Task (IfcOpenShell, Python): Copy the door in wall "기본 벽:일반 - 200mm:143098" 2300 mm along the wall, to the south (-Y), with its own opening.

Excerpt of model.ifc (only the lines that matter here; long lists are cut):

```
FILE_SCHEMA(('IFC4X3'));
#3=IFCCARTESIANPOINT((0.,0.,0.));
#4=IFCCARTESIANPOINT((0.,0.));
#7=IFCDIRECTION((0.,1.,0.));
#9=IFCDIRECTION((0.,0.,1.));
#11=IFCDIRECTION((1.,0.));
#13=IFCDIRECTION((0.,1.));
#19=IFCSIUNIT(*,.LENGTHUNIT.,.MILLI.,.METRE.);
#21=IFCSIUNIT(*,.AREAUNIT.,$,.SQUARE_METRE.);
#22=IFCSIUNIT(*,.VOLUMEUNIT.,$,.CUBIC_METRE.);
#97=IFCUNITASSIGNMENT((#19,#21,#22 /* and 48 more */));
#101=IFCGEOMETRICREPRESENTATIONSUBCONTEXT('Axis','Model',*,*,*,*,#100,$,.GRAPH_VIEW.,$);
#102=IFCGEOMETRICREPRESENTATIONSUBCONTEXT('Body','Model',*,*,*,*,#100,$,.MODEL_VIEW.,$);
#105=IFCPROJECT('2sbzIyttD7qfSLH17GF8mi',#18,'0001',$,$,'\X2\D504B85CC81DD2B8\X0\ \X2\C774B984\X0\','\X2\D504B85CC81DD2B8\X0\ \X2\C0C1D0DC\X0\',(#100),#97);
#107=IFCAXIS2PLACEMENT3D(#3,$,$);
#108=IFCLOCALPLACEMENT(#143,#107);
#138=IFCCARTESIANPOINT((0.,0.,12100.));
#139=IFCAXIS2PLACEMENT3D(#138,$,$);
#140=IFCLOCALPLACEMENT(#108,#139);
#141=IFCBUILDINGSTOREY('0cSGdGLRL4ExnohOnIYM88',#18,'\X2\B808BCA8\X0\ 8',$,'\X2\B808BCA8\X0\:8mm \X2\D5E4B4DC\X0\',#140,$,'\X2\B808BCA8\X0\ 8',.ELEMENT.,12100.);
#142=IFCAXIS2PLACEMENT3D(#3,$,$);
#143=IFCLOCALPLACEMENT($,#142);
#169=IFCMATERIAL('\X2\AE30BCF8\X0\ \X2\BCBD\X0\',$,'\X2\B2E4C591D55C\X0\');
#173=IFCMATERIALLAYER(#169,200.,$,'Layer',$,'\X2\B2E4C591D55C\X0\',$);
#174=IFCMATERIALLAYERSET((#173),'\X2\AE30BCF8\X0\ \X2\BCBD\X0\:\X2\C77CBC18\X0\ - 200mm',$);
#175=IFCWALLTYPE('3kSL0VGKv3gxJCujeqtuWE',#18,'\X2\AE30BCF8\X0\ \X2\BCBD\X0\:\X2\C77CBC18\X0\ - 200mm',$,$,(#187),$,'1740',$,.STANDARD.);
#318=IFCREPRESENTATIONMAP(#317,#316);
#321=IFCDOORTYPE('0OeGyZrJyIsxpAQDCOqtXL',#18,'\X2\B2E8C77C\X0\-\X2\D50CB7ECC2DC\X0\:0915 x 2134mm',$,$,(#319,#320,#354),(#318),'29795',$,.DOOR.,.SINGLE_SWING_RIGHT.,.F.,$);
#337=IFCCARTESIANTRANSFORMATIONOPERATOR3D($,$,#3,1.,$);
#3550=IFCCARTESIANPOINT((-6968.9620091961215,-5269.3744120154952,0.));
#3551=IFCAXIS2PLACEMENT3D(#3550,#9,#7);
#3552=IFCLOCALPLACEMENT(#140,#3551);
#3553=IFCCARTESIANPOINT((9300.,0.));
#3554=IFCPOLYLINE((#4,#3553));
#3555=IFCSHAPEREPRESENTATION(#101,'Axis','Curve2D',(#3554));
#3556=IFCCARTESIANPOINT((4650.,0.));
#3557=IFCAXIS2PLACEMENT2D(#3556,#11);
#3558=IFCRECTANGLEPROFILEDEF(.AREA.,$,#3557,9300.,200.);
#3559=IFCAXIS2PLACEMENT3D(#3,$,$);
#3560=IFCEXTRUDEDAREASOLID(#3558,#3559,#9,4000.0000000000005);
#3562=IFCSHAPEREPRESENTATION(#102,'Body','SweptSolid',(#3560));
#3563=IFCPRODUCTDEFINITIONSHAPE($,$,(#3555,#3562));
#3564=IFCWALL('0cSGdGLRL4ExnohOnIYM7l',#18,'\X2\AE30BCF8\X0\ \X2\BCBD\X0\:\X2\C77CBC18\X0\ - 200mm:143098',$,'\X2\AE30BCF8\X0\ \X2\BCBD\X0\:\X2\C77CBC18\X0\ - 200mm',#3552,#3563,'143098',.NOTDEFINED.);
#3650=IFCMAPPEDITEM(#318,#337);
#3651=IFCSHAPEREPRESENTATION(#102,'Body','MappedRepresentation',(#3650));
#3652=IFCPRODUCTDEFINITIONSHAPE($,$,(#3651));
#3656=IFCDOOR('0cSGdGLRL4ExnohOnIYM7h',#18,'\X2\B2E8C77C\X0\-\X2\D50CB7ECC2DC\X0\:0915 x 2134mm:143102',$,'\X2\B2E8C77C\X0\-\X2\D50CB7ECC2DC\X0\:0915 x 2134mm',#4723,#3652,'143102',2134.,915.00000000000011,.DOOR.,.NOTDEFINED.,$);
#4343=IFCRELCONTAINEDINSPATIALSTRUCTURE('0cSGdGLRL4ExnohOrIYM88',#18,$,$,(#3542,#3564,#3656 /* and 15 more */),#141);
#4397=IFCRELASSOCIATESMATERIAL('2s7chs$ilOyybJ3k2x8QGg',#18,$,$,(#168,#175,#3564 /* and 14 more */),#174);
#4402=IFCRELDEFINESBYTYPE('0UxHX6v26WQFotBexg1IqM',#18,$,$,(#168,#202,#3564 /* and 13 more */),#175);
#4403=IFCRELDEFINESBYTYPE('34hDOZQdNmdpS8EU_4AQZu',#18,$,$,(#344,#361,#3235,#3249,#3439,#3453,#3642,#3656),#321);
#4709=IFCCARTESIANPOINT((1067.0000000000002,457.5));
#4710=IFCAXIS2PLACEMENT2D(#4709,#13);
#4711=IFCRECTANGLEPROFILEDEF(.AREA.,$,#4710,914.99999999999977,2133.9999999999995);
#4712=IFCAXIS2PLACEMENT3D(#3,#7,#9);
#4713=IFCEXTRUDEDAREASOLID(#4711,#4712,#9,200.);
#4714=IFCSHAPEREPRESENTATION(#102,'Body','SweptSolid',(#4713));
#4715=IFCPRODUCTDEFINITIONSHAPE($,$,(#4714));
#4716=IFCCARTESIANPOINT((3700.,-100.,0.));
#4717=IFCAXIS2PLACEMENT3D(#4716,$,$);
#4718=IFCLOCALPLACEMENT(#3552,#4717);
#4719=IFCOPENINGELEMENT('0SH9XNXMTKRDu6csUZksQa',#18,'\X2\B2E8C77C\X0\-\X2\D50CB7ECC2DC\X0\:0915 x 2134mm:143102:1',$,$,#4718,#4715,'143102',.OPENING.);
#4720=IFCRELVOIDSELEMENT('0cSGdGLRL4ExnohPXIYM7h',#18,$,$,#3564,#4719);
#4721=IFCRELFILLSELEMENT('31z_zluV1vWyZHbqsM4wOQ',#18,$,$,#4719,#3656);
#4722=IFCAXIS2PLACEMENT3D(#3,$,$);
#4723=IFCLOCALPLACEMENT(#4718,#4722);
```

```python
import ifcopenshell
import ifcopenshell.api.feature
import ifcopenshell.api.geometry
import ifcopenshell.api.root
import ifcopenshell.geom
import ifcopenshell.util.element
import ifcopenshell.util.placement
import ifcopenshell.util.shape
import ifcopenshell.util.unit

model = ifcopenshell.open("model.ifc")
unit_scale = ifcopenshell.util.unit.calculate_unit_scale(model)
settings = ifcopenshell.geom.settings()


def volume(element):
    """Net volume in cubic metres, openings subtracted."""
    shape = ifcopenshell.geom.create_shape(settings, element)
    return ifcopenshell.util.shape.get_volume(shape.geometry)


def reuse_history(source, copy):
    """copy_class also copies each property set's owner history, people and application; keep the originals."""
    for rel in copy.IsDefinedBy:
        if rel.is_a("IfcRelDefinesByProperties") and (history := rel.RelatingPropertyDefinition.OwnerHistory):
            rel.RelatingPropertyDefinition.OwnerHistory = source.OwnerHistory
            ifcopenshell.util.element.remove_deep2(model, history)


door = model.by_id(3656)
opening = door.FillsVoids[0].RelatingOpeningElement
wall = opening.VoidsElements[0].RelatingBuildingElement
before = volume(wall)
shift = ifcopenshell.util.placement.get_local_placement(wall.ObjectPlacement)[:3, 0] * -2.3 / unit_scale

# copy_class copies the void relationship, type, container and properties, but no geometry.
new_opening = ifcopenshell.api.root.copy_class(model, product=opening)
new_opening.Representation = ifcopenshell.util.element.copy_deep(
    model, opening.Representation, exclude=["IfcGeometricRepresentationContext", "IfcRepresentationMap"]
)
new_opening.Name = "단일-플러시:0915 x 2134mm"
new_opening.Tag = None
new_door = ifcopenshell.api.root.copy_class(model, product=door)
new_door.Representation = ifcopenshell.util.element.copy_deep(
    model, door.Representation, exclude=["IfcGeometricRepresentationContext", "IfcRepresentationMap"]
)
new_door.Name = "단일-플러시:0915 x 2134mm"
new_door.Tag = None
reuse_history(door, new_door)
ifcopenshell.api.feature.add_filling(model, opening=new_opening, element=new_door)

for old, new in ((opening, new_opening), (door, new_door)):
    matrix = ifcopenshell.util.placement.get_local_placement(old.ObjectPlacement)
    matrix[:3, 3] += shift
    ifcopenshell.api.geometry.edit_object_placement(model, product=new, matrix=matrix, is_si=False)

after = volume(wall)

print(f"wall volume {before:.3f} -> {after:.3f} m3")

model.write("model_edited.ifc")
```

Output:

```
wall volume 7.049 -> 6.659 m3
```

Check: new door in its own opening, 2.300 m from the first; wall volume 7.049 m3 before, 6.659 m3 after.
